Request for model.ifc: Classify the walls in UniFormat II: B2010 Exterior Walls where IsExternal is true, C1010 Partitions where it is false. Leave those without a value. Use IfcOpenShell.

First a look at what the model holds.

```python
import ifcopenshell
import ifcopenshell.util.element

model = ifcopenshell.open("model.ifc")
print(model.schema)
print("classifications:", [c.Name for c in model.by_type("IfcClassification")])
values = [ifcopenshell.util.element.get_pset(e, "Pset_WallCommon", "IsExternal") for e in model.by_type("IfcWall")]
for value in (True, False, None):
    print("IsExternal", value, values.count(value))
```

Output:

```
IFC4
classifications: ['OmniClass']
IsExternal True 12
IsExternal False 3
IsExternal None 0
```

```python
import ifcopenshell
import ifcopenshell.api.classification
import ifcopenshell.util.element

model = ifcopenshell.open("model.ifc")

system = ifcopenshell.api.classification.add_classification(model, classification="UniFormat II")

walls = model.by_type("IfcWall")
external = {e: ifcopenshell.util.element.get_pset(e, "Pset_WallCommon", "IsExternal") for e in walls}
for flag, code, name in ((True, "B2010", "Exterior Walls"), (False, "C1010", "Partitions")):
    products = [e for e in walls if external[e] is flag]
    ifcopenshell.api.classification.add_reference(
        model, products=products, classification=system, identification=code, name=name
    )
    print(code, len(products))

model.write("model-out.ifc")
```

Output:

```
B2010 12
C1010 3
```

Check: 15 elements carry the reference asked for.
